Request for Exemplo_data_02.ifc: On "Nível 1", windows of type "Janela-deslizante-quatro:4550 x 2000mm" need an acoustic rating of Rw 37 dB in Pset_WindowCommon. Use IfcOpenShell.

First a look at what the model holds.

```python
import ifcopenshell
import ifcopenshell.util.element

model = ifcopenshell.open("Exemplo_data_02.ifc")
print(model.schema)
storey = next(s for s in model.by_type("IfcBuildingStorey") if s.Name == "Nível 1")
windows = [e for e in ifcopenshell.util.element.get_decomposition(storey) if e.is_a("IfcWindow")]
seen = {}
for e in windows:
    element_type = ifcopenshell.util.element.get_type(e)
    key = (element_type.Name if element_type != e and element_type else None, ifcopenshell.util.element.get_pset(e, "Pset_WindowCommon", "AcousticRating"))
    seen[key] = seen.get(key, 0) + 1
for (name, value), count in sorted(seen.items(), key=str):
    print(count, "x", name, "|", value)
```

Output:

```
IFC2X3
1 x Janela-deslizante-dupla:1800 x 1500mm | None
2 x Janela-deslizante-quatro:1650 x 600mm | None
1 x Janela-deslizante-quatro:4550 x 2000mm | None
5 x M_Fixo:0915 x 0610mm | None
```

```python
import ifcopenshell
import ifcopenshell.api.pset
import ifcopenshell.util.element

model = ifcopenshell.open("Exemplo_data_02.ifc")

storey = next(s for s in model.by_type("IfcBuildingStorey") if s.Name == "Nível 1")
windows = [e for e in ifcopenshell.util.element.get_decomposition(storey) if e.is_a("IfcWindow")]

count = 0
for e in windows:
    element_type = ifcopenshell.util.element.get_type(e)
    if element_type in (None, e) or element_type.Name != "Janela-deslizante-quatro:4550 x 2000mm":
        continue
    # add_pset returns the element's existing set when there is one.
    pset = ifcopenshell.api.pset.add_pset(model, product=e, name="Pset_WindowCommon")
    ifcopenshell.api.pset.edit_pset(model, pset=pset, properties={"AcousticRating": "Rw 37 dB"})
    count += 1

print(count, "windows updated")

model.write("Exemplo_data_02-out.ifc")
```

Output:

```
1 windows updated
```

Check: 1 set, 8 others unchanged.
